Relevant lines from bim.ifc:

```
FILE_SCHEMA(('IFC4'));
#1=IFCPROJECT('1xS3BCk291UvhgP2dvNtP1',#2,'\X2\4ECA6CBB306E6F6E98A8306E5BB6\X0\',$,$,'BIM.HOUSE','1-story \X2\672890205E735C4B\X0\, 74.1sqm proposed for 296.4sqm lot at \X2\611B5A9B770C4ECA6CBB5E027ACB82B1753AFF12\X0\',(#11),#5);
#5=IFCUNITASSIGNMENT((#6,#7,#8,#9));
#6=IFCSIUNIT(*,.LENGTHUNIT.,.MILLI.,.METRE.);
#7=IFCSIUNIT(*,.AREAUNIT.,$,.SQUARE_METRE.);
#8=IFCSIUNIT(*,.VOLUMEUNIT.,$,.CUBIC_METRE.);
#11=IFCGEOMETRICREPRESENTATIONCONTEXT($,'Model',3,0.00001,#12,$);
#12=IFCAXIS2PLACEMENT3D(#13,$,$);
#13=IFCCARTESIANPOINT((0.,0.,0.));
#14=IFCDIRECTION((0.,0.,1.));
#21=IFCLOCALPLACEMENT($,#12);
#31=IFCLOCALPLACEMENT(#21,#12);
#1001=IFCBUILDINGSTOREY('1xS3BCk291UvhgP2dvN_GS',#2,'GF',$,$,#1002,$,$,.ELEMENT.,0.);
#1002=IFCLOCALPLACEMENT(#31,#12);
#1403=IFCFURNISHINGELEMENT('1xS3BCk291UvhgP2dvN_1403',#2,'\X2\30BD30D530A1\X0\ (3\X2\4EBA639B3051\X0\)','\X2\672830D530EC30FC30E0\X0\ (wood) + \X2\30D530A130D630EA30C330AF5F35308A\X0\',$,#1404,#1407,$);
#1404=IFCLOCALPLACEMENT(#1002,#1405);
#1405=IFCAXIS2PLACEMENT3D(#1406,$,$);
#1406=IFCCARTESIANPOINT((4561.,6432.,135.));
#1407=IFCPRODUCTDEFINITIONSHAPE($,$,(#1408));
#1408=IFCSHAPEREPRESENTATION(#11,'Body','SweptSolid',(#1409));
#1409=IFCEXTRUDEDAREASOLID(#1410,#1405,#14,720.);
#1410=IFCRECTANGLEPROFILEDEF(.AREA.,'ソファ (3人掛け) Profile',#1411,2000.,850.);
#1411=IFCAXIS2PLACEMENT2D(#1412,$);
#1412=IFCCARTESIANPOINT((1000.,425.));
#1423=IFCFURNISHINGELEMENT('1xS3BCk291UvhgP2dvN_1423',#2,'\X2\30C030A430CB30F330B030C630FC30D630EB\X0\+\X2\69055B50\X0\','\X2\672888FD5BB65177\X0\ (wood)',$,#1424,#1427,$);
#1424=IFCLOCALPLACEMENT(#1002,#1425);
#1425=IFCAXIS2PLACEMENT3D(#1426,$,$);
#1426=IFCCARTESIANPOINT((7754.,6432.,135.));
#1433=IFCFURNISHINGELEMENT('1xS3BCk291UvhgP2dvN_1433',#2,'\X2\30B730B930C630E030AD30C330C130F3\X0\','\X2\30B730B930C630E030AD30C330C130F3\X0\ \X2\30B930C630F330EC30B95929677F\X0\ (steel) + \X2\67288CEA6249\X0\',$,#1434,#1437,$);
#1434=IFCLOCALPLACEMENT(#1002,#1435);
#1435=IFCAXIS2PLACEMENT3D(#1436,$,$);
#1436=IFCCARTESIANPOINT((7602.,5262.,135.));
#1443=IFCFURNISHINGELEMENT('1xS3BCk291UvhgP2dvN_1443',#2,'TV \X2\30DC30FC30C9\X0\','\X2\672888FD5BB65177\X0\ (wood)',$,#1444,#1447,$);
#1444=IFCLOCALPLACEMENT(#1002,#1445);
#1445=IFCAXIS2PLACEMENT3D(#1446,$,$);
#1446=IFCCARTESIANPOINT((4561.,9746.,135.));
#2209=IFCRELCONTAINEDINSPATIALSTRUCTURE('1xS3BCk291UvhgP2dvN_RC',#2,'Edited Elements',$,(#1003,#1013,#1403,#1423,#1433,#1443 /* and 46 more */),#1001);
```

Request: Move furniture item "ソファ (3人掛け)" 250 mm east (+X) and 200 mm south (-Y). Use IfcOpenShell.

```python
import ifcopenshell
import ifcopenshell.api.geometry
import ifcopenshell.util.placement
import ifcopenshell.util.unit

model = ifcopenshell.open("bim.ifc")
unit_scale = ifcopenshell.util.unit.calculate_unit_scale(model)

item = model.by_guid("1xS3BCk291UvhgP2dvN_1403")
matrix = ifcopenshell.util.placement.get_local_placement(item.ObjectPlacement)
matrix[0, 3] += 0.25 / unit_scale
matrix[1, 3] -= 0.2 / unit_scale
ifcopenshell.api.geometry.edit_object_placement(model, product=item, matrix=matrix, is_si=False)

print(ifcopenshell.util.placement.get_local_placement(item.ObjectPlacement).round(3) + 0.0)

model.write("bim_rev.ifc")
```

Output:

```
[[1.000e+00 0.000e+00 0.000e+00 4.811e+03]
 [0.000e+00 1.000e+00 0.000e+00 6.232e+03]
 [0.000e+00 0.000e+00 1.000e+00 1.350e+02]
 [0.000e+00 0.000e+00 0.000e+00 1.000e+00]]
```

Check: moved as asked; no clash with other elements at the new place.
